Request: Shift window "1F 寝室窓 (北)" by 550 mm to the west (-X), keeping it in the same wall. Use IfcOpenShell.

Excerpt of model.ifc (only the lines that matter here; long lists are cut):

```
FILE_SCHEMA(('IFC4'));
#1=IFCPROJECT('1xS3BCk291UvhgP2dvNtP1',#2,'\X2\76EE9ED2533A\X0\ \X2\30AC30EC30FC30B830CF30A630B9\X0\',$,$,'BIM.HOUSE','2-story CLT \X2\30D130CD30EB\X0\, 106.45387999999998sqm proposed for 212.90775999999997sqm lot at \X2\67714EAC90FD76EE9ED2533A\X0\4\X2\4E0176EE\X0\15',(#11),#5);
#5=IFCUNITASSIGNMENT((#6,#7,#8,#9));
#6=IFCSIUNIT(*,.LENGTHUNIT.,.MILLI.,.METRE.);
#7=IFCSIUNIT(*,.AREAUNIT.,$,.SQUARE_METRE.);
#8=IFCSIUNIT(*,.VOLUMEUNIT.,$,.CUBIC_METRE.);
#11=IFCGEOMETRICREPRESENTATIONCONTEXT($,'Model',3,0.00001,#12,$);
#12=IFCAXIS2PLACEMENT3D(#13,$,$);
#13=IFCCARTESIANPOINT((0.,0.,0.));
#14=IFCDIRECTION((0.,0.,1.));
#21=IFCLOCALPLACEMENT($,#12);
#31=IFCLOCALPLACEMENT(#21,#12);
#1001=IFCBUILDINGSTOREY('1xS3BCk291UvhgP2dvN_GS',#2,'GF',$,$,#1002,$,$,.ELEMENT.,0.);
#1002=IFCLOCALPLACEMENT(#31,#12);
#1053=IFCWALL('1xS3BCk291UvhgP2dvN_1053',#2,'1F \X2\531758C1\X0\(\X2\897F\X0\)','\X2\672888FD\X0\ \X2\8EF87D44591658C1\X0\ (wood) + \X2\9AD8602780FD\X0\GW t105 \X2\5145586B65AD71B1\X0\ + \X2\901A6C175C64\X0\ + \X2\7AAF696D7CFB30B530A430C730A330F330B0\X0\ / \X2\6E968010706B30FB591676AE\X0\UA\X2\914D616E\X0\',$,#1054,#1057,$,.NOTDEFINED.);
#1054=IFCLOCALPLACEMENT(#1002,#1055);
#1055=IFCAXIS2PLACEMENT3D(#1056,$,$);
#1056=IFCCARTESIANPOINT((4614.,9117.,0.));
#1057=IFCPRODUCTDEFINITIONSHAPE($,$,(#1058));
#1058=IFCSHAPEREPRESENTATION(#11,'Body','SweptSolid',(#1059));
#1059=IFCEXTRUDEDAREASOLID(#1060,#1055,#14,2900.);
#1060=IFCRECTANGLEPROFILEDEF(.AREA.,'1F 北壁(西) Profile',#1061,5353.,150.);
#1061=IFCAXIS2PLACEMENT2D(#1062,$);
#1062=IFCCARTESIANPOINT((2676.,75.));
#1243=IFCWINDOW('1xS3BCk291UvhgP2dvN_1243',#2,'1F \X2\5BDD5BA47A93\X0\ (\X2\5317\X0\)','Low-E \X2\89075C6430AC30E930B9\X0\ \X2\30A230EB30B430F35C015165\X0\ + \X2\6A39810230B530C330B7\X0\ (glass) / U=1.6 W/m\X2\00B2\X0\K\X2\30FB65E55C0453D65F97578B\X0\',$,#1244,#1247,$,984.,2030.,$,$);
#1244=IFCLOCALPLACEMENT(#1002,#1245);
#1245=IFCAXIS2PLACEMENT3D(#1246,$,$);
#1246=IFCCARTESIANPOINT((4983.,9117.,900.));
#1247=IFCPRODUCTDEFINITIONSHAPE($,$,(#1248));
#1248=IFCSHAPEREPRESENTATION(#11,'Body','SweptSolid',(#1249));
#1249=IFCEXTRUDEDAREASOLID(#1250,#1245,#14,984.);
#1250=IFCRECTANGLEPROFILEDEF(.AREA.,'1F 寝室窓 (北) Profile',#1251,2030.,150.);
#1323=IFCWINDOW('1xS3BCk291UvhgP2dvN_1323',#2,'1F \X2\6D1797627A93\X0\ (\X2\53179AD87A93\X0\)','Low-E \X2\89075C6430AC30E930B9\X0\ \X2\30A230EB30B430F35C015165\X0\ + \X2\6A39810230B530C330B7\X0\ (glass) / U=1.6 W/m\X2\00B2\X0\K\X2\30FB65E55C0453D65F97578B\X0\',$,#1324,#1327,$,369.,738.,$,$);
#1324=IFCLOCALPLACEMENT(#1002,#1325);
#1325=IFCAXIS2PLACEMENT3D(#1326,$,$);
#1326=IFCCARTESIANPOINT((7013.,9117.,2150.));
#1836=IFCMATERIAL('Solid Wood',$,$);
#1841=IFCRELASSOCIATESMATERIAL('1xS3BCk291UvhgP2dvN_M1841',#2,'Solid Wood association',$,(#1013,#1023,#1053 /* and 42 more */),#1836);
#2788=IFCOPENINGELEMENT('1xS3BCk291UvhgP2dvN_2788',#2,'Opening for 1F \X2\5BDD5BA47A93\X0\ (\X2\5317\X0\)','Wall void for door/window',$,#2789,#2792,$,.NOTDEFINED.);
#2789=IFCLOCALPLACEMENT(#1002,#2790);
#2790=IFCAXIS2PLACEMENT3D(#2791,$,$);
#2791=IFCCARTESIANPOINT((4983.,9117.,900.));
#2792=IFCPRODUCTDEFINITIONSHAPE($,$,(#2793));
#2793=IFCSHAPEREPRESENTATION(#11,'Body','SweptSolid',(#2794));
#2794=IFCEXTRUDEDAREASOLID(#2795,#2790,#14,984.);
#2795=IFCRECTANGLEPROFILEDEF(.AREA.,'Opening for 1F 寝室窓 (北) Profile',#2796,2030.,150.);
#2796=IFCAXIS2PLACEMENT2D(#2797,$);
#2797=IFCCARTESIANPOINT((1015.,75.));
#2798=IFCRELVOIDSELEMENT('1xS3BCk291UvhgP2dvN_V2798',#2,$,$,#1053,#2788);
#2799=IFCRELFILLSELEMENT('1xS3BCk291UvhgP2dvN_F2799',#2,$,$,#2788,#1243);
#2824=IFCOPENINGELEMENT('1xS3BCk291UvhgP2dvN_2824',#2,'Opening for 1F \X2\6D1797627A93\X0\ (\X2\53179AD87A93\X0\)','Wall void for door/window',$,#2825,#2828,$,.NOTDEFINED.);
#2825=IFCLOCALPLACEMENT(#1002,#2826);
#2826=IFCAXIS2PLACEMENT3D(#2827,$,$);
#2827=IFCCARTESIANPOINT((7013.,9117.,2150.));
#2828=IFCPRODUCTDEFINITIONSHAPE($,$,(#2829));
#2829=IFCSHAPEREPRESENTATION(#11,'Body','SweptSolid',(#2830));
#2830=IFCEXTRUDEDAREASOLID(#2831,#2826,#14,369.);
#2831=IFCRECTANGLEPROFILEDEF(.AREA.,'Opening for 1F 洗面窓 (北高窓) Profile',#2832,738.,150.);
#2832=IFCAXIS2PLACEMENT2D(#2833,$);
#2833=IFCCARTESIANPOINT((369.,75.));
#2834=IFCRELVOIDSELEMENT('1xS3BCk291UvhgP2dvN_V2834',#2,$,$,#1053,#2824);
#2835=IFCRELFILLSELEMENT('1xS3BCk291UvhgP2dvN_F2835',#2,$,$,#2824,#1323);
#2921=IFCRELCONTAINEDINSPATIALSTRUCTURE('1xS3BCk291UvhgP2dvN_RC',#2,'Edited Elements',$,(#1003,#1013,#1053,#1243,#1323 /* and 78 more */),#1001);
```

```python
import ifcopenshell
import ifcopenshell.api.geometry
import ifcopenshell.util.placement
import ifcopenshell.util.unit

model = ifcopenshell.open("model.ifc")
unit_scale = ifcopenshell.util.unit.calculate_unit_scale(model)

window = model.by_guid("1xS3BCk291UvhgP2dvN_1243")
opening = window.FillsVoids[0].RelatingOpeningElement
wall = opening.VoidsElements[0].RelatingBuildingElement

wall_matrix = ifcopenshell.util.placement.get_local_placement(wall.ObjectPlacement)
shift = wall_matrix[:3, 0] * -0.55 / unit_scale
before = ifcopenshell.util.placement.get_local_placement(window.ObjectPlacement)[:3, 3].copy()

# The window is not placed relative to its opening, so move both.
for product in (opening, window):
    matrix = ifcopenshell.util.placement.get_local_placement(product.ObjectPlacement)
    matrix[:3, 3] += shift
    ifcopenshell.api.geometry.edit_object_placement(model, product=product, matrix=matrix, is_si=False)

after = ifcopenshell.util.placement.get_local_placement(window.ObjectPlacement)[:3, 3]
print("window moved by", (after - before).round(3) + 0.0)

model.write("model_updated.ifc")
```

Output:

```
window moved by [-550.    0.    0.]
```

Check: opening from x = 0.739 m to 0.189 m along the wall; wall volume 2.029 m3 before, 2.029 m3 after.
